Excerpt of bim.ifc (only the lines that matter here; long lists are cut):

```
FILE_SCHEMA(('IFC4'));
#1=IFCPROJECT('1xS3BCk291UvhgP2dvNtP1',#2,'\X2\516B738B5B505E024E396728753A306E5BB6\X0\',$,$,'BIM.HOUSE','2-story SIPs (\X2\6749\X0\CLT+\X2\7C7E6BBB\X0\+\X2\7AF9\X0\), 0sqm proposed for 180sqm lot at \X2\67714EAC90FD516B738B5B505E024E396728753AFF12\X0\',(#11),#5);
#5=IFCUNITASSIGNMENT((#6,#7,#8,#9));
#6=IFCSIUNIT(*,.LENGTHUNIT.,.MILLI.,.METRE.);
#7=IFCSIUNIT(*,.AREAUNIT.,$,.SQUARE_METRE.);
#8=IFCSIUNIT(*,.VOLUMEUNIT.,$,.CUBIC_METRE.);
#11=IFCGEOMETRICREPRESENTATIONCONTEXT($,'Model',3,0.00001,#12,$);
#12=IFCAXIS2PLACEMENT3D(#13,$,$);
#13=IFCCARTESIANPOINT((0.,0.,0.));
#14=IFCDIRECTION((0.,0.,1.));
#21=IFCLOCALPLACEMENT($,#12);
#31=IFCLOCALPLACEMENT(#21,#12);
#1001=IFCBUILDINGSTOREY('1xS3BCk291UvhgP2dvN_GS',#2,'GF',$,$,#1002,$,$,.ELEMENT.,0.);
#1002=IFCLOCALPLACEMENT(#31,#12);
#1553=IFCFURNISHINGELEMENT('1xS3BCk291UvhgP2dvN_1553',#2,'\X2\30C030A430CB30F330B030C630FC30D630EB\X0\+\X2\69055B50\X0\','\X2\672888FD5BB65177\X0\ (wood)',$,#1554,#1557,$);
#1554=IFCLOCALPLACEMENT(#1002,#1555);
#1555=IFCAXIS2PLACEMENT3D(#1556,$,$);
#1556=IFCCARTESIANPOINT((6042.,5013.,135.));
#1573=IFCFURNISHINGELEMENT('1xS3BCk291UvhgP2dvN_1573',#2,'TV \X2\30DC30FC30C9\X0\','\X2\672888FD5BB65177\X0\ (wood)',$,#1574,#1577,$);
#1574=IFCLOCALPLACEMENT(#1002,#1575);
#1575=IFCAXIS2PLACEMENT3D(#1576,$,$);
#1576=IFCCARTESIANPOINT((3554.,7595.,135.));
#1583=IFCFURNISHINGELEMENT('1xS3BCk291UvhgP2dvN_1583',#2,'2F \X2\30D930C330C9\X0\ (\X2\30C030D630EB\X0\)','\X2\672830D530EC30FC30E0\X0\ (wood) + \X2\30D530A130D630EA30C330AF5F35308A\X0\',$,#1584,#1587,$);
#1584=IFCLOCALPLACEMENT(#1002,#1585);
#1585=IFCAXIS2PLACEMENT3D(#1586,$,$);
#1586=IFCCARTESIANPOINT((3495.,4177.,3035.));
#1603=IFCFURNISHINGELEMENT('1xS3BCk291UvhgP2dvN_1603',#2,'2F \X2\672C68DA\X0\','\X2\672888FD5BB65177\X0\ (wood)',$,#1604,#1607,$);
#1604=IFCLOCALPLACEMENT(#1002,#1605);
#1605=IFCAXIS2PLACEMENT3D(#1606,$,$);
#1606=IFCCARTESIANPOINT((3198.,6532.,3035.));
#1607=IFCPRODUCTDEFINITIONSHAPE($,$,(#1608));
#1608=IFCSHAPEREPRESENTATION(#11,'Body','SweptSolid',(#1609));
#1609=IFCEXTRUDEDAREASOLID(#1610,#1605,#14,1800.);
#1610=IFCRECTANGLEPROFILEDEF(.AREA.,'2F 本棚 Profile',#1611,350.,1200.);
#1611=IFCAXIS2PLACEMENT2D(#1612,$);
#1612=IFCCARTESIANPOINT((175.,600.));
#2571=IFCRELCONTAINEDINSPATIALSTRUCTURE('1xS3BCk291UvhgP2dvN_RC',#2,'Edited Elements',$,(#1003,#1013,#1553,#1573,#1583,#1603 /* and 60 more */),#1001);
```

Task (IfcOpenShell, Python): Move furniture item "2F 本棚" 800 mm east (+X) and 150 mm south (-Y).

```python
import ifcopenshell
import ifcopenshell.api.geometry
import ifcopenshell.util.placement

model = ifcopenshell.open("bim.ifc")

item = model.by_guid("1xS3BCk291UvhgP2dvN_1603")
matrix = ifcopenshell.util.placement.get_local_placement(item.ObjectPlacement)
matrix[0, 3] += 800.0
matrix[1, 3] -= 150.0
ifcopenshell.api.geometry.edit_object_placement(model, product=item, matrix=matrix, is_si=False)

print(ifcopenshell.util.placement.get_local_placement(item.ObjectPlacement).round(3) + 0.0)

model.write("bim_rev.ifc")
```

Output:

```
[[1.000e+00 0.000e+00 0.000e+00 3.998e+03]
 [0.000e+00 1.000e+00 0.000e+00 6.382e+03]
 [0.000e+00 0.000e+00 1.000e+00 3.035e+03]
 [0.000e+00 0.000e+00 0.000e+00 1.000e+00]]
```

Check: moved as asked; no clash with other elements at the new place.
